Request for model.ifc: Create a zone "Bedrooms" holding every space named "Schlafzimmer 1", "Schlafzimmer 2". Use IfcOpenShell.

First a look at what the model holds.

```python
import ifcopenshell

model = ifcopenshell.open("model.ifc")
print(model.schema)
seen = {}
for space in model.by_type("IfcSpace"):
    seen[space.LongName] = seen.get(space.LongName, 0) + 1
for name, count in sorted(seen.items(), key=str):
    print(count, "x", name)
print("zones:", [z.Name for z in model.by_type("IfcZone")][:20])
```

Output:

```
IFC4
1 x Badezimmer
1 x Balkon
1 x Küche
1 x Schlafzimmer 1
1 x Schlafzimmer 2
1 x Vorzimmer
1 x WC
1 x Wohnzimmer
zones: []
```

```python
import ifcopenshell
import ifcopenshell.api.group
import ifcopenshell.api.root

model = ifcopenshell.open("model.ifc")

names = {"Schlafzimmer 1", "Schlafzimmer 2"}
spaces = [s for s in model.by_type("IfcSpace") if s.LongName in names]

zone = ifcopenshell.api.root.create_entity(model, ifc_class="IfcZone", name="Bedrooms")
ifcopenshell.api.group.assign_group(model, products=spaces, group=zone)
print(len(spaces), "spaces in", zone.Name)

model.write("model_updated.ifc")
```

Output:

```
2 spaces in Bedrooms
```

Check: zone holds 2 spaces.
